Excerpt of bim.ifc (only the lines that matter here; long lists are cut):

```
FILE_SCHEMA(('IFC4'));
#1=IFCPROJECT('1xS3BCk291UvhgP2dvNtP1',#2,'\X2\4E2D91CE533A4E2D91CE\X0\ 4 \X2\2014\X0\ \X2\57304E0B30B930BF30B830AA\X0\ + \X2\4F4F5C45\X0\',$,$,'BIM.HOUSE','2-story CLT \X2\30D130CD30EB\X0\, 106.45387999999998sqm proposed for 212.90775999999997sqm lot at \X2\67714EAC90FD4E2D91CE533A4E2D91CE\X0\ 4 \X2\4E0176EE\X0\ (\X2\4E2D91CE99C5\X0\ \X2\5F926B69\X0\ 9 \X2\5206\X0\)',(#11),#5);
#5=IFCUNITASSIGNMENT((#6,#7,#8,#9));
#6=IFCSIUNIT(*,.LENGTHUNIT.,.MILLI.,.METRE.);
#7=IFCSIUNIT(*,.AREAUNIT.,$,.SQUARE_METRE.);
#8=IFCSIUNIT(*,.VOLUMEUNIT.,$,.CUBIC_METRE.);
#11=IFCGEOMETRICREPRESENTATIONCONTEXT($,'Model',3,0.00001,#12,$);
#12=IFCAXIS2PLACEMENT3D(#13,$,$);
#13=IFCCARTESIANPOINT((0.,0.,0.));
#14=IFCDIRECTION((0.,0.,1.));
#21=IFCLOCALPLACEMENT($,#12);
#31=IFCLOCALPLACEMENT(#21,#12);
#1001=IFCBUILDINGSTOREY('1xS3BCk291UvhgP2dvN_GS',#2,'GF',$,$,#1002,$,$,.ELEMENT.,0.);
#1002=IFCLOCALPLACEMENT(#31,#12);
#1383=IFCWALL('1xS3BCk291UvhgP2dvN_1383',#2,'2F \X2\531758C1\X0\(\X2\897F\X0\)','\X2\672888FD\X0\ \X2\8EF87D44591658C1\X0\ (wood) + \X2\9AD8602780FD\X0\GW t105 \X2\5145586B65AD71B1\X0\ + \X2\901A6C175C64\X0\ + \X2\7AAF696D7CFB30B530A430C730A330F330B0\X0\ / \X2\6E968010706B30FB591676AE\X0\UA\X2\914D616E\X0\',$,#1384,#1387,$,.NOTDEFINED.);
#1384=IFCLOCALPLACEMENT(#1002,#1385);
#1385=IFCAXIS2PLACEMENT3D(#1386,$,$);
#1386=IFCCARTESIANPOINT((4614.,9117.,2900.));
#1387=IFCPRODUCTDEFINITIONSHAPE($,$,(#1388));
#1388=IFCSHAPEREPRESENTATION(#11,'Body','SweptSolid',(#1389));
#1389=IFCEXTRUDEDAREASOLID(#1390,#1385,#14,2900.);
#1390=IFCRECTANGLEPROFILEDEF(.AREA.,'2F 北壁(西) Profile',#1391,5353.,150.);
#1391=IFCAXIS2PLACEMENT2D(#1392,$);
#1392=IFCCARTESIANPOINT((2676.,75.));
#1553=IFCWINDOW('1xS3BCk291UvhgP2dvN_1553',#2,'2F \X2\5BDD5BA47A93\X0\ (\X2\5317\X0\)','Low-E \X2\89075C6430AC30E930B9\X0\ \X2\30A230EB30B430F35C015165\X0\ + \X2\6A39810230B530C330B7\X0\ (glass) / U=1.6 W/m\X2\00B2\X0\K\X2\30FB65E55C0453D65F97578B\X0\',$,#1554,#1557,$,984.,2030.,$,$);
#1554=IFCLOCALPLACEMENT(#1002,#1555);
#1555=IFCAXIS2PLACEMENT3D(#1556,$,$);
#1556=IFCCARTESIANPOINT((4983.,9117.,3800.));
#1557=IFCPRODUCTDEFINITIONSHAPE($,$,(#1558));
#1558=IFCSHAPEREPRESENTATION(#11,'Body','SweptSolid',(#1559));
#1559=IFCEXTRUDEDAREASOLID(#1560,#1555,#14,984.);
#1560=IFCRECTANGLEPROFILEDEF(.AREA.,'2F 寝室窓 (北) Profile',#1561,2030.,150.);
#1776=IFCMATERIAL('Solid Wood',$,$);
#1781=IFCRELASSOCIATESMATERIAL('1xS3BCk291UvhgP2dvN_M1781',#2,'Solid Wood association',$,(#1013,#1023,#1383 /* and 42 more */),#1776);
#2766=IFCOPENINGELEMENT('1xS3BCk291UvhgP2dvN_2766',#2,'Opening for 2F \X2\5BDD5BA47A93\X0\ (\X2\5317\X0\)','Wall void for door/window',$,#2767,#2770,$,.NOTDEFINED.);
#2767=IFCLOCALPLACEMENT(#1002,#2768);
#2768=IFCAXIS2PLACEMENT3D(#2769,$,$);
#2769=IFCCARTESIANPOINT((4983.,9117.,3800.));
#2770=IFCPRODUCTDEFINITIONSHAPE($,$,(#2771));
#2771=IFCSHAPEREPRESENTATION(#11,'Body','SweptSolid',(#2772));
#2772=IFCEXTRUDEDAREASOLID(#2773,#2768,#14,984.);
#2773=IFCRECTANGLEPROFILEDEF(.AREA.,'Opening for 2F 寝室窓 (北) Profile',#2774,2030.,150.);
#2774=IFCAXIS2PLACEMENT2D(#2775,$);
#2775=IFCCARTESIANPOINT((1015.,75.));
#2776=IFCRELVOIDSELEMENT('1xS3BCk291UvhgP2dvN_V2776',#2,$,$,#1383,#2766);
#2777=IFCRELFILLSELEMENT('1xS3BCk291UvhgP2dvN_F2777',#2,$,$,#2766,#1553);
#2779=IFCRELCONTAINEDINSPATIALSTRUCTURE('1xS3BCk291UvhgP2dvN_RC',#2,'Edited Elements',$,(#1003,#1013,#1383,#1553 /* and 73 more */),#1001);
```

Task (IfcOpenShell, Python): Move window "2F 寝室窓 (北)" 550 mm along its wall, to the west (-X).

```python
import ifcopenshell
import ifcopenshell.api.geometry
import ifcopenshell.util.placement
import ifcopenshell.util.unit

model = ifcopenshell.open("bim.ifc")
unit_scale = ifcopenshell.util.unit.calculate_unit_scale(model)

window = model.by_guid("1xS3BCk291UvhgP2dvN_1553")
opening = window.FillsVoids[0].RelatingOpeningElement
wall = opening.VoidsElements[0].RelatingBuildingElement

wall_matrix = ifcopenshell.util.placement.get_local_placement(wall.ObjectPlacement)
shift = wall_matrix[:3, 0] * -0.55 / unit_scale
before = ifcopenshell.util.placement.get_local_placement(window.ObjectPlacement)[:3, 3].copy()

# The window is not placed relative to its opening, so move both.
for product in (opening, window):
    matrix = ifcopenshell.util.placement.get_local_placement(product.ObjectPlacement)
    matrix[:3, 3] += shift
    ifcopenshell.api.geometry.edit_object_placement(model, product=product, matrix=matrix, is_si=False)

after = ifcopenshell.util.placement.get_local_placement(window.ObjectPlacement)[:3, 3]
print("window moved by", (after - before).round(3) + 0.0)

model.write("bim_edited.ifc")
```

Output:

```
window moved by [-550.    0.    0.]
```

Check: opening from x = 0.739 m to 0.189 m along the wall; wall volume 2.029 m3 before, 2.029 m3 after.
